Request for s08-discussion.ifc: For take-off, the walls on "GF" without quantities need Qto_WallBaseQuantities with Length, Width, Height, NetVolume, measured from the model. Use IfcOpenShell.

First a look at what the model holds.

```python
import ifcopenshell
import ifcopenshell.util.element
import ifcopenshell.util.unit

model = ifcopenshell.open("s08-discussion.ifc")
print(model.schema)
for unit_type in ("LENGTHUNIT", "AREAUNIT", "VOLUMEUNIT"):
    print(unit_type, ifcopenshell.util.unit.calculate_unit_scale(model, unit_type))
storey = next(s for s in model.by_type("IfcBuildingStorey") if s.Name == "GF")
walls = [e for e in ifcopenshell.util.element.get_decomposition(storey) if e.is_a("IfcWall")]
for e in sorted(walls, key=lambda e: e.id()):
    print(e.id(), e.is_a(), e.Name, list(ifcopenshell.util.element.get_psets(e, qtos_only=True)), sep=" | ")
```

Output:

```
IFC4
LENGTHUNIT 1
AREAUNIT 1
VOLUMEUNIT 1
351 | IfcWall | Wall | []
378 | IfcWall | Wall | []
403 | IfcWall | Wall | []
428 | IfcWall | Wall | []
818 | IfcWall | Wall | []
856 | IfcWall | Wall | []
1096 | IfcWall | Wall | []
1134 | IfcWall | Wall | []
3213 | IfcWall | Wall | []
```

```python
import ifcopenshell
import ifcopenshell.api.pset
import ifcopenshell.geom
import ifcopenshell.util.element
import ifcopenshell.util.shape
import ifcopenshell.util.unit

model = ifcopenshell.open("s08-discussion.ifc")
unit_scale = ifcopenshell.util.unit.calculate_unit_scale(model)
volume_scale = ifcopenshell.util.unit.calculate_unit_scale(model, "VOLUMEUNIT")
settings = ifcopenshell.geom.settings()

storey = next(s for s in model.by_type("IfcBuildingStorey") if s.Name == "GF")
walls = [e for e in ifcopenshell.util.element.get_decomposition(storey) if e.is_a("IfcWall")]

for e in sorted(walls, key=lambda e: e.id()):
    if ifcopenshell.util.element.get_psets(e, qtos_only=True, should_inherit=False):
        continue
    # Geometry comes back in metres, in the element's own axes.
    shape = ifcopenshell.geom.create_shape(settings, e)
    values = {
        "Length": ifcopenshell.util.shape.get_x(shape.geometry) / unit_scale,
        "Width": ifcopenshell.util.shape.get_y(shape.geometry) / unit_scale,
        "Height": ifcopenshell.util.shape.get_z(shape.geometry) / unit_scale,
        "NetVolume": ifcopenshell.util.shape.get_volume(shape.geometry) / volume_scale,
    }
    qto = ifcopenshell.api.pset.add_qto(model, product=e, name="Qto_WallBaseQuantities")
    ifcopenshell.api.pset.edit_qto(model, qto=qto, properties=values)
    print(e.id(), {k: round(v, 3) for k, v in values.items()})

model.write("s08-discussion_updated.ifc")
```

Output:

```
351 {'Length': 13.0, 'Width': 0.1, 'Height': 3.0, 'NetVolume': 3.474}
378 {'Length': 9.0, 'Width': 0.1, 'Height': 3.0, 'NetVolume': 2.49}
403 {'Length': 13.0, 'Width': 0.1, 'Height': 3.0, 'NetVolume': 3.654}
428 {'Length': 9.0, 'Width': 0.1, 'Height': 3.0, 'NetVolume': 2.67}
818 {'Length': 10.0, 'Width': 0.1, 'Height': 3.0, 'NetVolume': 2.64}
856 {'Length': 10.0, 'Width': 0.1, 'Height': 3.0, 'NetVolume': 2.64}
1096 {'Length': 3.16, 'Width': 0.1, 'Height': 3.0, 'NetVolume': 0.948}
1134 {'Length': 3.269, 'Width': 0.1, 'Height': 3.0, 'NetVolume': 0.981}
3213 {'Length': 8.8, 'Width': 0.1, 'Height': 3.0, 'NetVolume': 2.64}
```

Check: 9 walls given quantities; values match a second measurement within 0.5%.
